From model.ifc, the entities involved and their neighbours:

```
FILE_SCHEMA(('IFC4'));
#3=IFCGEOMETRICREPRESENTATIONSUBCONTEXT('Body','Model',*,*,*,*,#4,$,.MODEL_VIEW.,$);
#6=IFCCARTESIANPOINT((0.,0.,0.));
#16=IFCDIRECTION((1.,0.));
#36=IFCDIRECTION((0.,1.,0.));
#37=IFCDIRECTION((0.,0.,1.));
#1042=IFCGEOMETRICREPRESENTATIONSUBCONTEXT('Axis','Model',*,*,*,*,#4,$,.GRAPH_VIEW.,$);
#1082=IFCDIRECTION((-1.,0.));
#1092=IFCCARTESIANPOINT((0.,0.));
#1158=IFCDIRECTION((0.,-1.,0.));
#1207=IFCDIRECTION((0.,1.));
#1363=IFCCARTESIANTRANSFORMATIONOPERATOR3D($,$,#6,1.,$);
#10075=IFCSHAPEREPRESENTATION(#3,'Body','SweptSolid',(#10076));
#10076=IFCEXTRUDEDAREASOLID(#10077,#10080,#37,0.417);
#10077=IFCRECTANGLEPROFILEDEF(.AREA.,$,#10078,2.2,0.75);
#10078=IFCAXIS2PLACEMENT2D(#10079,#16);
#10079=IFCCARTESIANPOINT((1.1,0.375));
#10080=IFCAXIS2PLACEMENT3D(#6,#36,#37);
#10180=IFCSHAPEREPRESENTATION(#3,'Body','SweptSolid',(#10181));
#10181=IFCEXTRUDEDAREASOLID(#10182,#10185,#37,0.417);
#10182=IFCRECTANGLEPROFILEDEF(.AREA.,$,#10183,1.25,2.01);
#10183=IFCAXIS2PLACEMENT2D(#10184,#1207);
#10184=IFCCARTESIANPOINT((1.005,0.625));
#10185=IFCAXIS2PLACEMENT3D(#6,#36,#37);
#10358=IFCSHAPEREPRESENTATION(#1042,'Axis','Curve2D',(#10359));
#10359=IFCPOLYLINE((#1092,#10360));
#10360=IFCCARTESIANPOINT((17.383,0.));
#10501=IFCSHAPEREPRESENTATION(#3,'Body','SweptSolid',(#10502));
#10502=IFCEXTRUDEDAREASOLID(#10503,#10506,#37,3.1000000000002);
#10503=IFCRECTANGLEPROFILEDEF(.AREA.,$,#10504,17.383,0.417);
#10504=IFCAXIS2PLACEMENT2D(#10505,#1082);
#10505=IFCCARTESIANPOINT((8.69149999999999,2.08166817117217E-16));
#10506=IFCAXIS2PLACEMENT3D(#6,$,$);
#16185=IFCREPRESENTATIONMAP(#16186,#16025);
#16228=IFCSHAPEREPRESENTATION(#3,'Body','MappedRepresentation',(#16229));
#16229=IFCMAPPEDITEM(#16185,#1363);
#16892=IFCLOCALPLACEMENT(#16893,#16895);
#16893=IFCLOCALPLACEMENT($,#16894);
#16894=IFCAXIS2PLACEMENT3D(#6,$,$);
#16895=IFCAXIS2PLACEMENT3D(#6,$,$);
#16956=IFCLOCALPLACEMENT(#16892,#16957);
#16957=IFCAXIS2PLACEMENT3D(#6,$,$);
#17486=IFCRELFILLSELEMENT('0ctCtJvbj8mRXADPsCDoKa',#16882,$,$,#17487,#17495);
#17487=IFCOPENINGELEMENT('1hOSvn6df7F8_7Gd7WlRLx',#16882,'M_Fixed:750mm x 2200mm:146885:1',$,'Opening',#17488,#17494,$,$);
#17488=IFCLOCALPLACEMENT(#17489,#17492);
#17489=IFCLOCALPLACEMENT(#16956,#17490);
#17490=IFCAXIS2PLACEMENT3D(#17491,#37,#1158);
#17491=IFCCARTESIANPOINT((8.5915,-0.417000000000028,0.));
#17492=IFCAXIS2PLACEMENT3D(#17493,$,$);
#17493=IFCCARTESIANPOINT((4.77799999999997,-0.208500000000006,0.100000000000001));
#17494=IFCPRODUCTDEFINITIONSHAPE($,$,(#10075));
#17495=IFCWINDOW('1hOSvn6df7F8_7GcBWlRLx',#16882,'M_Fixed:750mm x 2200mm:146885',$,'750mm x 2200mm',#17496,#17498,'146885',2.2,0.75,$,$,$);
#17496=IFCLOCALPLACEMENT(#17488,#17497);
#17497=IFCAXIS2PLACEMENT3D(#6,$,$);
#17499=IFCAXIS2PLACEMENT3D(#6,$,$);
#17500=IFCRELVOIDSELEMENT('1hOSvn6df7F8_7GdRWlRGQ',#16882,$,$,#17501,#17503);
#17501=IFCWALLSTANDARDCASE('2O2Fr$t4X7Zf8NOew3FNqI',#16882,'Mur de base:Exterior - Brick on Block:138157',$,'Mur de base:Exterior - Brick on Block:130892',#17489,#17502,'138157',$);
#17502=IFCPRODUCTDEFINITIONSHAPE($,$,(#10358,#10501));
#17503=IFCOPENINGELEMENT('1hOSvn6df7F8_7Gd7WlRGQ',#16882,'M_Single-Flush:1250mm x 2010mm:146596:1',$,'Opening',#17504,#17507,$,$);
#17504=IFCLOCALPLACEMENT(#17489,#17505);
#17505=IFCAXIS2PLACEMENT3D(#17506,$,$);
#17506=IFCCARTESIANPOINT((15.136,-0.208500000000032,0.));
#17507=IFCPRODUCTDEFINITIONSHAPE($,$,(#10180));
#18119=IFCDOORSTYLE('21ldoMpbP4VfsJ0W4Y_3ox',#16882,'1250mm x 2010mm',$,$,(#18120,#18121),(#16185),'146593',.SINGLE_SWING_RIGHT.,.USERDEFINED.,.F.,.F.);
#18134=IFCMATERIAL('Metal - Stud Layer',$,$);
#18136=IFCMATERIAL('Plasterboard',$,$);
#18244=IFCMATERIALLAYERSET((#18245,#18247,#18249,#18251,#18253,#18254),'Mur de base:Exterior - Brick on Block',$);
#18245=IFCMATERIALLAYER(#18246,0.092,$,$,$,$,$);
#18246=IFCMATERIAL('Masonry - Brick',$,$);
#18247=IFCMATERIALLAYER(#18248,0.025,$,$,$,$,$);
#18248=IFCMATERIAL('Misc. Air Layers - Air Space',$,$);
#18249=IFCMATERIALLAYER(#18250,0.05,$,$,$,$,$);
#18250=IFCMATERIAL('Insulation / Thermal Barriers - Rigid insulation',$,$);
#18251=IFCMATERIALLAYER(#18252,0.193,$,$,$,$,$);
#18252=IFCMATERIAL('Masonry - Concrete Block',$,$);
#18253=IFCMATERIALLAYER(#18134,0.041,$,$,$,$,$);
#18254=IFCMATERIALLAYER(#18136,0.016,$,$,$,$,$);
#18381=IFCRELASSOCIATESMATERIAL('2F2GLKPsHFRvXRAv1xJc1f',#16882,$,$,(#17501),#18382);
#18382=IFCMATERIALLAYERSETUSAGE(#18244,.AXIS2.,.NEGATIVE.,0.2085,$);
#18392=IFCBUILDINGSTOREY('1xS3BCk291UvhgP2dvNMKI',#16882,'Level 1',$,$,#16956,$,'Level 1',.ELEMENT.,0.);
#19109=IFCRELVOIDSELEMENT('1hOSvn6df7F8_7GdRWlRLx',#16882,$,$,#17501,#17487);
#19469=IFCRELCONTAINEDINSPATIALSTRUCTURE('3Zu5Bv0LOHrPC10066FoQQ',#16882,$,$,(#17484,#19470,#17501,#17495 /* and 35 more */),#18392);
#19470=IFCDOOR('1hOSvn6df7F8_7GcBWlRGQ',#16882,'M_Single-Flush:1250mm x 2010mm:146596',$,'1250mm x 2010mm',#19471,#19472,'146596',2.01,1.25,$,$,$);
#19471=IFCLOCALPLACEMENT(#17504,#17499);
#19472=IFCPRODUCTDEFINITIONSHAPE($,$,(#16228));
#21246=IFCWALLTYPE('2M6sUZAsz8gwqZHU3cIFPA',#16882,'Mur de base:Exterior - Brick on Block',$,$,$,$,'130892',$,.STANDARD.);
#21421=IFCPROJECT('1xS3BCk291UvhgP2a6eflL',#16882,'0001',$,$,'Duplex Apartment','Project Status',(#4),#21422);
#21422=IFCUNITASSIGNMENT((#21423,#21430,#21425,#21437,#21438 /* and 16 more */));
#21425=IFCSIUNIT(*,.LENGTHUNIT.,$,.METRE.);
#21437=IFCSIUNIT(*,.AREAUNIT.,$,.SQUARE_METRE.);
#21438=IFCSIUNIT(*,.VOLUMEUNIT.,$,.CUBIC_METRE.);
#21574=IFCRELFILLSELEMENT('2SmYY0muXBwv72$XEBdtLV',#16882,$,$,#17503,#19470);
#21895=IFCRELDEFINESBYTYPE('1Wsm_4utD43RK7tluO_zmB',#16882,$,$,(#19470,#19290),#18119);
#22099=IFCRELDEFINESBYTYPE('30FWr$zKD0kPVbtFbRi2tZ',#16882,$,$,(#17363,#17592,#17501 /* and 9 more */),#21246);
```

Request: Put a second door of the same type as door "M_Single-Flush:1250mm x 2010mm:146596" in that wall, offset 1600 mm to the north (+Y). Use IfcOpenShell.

```python
import ifcopenshell
import ifcopenshell.api.feature
import ifcopenshell.api.geometry
import ifcopenshell.api.root
import ifcopenshell.geom
import ifcopenshell.util.element
import ifcopenshell.util.placement
import ifcopenshell.util.shape
import ifcopenshell.util.unit

model = ifcopenshell.open("model.ifc")
unit_scale = ifcopenshell.util.unit.calculate_unit_scale(model)
settings = ifcopenshell.geom.settings()


def volume(element):
    """Net volume in cubic metres, openings subtracted."""
    shape = ifcopenshell.geom.create_shape(settings, element)
    return ifcopenshell.util.shape.get_volume(shape.geometry)


def reuse_history(source, copy):
    """copy_class also copies each property set's owner history, people and application; keep the originals."""
    for rel in copy.IsDefinedBy:
        if rel.is_a("IfcRelDefinesByProperties") and (history := rel.RelatingPropertyDefinition.OwnerHistory):
            rel.RelatingPropertyDefinition.OwnerHistory = source.OwnerHistory
            ifcopenshell.util.element.remove_deep2(model, history)


door = model.by_id(19470)
opening = door.FillsVoids[0].RelatingOpeningElement
wall = opening.VoidsElements[0].RelatingBuildingElement
before = volume(wall)
shift = ifcopenshell.util.placement.get_local_placement(wall.ObjectPlacement)[:3, 0] * -1.6 / unit_scale

# copy_class copies the void relationship, type, container and properties, but no geometry.
new_opening = ifcopenshell.api.root.copy_class(model, product=opening)
new_opening.Representation = ifcopenshell.util.element.copy_deep(
    model, opening.Representation, exclude=["IfcGeometricRepresentationContext", "IfcRepresentationMap"]
)
new_opening.Name = "M_Single-Flush:1250mm x 2010mm"
new_door = ifcopenshell.api.root.copy_class(model, product=door)
new_door.Representation = ifcopenshell.util.element.copy_deep(
    model, door.Representation, exclude=["IfcGeometricRepresentationContext", "IfcRepresentationMap"]
)
new_door.Name = "M_Single-Flush:1250mm x 2010mm"
new_door.Tag = None
reuse_history(door, new_door)
ifcopenshell.api.feature.add_filling(model, opening=new_opening, element=new_door)

for old, new in ((opening, new_opening), (door, new_door)):
    matrix = ifcopenshell.util.placement.get_local_placement(old.ObjectPlacement)
    matrix[:3, 3] += shift
    ifcopenshell.api.geometry.edit_object_placement(model, product=new, matrix=matrix, is_si=False)

after = volume(wall)

print(f"wall volume {before:.3f} -> {after:.3f} m3")

model.write("model-out.ifc")
```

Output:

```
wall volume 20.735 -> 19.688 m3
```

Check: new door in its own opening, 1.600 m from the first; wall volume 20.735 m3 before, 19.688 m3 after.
